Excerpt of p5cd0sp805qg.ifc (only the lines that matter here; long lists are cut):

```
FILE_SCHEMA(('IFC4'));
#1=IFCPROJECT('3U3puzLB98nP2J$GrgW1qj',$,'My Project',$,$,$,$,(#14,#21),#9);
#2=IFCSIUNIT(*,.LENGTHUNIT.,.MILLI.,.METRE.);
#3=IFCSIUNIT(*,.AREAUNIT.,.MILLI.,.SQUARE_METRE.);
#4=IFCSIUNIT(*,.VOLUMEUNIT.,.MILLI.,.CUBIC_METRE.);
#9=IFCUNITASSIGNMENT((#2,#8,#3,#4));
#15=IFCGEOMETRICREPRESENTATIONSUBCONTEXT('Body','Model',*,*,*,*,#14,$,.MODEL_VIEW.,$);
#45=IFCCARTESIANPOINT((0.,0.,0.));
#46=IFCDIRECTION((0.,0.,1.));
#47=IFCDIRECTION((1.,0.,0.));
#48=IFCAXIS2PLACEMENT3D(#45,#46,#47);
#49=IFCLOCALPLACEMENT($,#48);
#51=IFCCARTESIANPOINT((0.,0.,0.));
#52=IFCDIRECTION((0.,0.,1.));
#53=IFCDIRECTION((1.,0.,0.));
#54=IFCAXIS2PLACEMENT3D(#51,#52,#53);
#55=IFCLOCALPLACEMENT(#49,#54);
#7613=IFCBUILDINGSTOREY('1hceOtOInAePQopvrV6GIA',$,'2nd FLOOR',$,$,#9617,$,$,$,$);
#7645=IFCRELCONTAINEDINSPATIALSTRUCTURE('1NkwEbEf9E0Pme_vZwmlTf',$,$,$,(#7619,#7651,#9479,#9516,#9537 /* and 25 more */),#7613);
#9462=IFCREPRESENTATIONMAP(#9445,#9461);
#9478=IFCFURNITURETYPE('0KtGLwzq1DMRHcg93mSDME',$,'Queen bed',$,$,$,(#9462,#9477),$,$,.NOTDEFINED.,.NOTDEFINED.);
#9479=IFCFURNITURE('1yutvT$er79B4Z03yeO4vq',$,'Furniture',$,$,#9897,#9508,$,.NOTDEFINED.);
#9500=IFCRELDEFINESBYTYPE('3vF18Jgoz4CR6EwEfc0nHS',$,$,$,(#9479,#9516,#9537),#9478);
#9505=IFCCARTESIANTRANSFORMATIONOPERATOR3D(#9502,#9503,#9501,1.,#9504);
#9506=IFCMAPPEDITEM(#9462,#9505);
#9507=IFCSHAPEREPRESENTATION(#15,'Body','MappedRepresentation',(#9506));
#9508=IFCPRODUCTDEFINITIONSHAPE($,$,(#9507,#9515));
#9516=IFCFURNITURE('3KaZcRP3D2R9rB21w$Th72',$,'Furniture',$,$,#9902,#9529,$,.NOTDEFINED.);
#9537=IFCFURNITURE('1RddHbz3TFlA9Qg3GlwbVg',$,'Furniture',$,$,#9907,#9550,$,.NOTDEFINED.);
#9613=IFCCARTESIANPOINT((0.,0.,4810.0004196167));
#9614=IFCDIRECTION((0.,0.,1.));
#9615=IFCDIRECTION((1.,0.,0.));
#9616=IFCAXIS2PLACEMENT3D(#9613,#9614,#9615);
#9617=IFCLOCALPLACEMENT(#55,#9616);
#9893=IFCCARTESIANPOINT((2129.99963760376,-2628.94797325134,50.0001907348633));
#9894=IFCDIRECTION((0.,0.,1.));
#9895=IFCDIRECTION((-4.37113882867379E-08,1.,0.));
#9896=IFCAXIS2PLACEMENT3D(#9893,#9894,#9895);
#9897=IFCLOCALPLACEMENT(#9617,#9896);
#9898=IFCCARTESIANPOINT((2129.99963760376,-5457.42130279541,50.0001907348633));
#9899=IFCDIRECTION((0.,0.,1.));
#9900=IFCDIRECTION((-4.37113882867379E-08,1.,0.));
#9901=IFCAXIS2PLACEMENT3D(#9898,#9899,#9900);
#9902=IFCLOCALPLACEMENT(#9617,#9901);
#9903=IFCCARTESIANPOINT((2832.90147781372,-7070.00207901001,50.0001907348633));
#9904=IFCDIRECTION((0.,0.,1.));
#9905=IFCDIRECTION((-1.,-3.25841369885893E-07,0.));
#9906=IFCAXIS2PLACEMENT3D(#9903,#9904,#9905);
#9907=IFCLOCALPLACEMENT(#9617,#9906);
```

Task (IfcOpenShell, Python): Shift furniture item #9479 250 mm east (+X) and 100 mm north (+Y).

```python
import ifcopenshell
import ifcopenshell.api.geometry
import ifcopenshell.util.placement
import ifcopenshell.util.unit

model = ifcopenshell.open("p5cd0sp805qg.ifc")
unit_scale = ifcopenshell.util.unit.calculate_unit_scale(model)

item = model.by_id(9479)
matrix = ifcopenshell.util.placement.get_local_placement(item.ObjectPlacement)
matrix[0, 3] += 0.25 / unit_scale
matrix[1, 3] += 0.1 / unit_scale
ifcopenshell.api.geometry.edit_object_placement(model, product=item, matrix=matrix, is_si=False)

print(ifcopenshell.util.placement.get_local_placement(item.ObjectPlacement).round(3) + 0.0)

model.write("p5cd0sp805qg_v2.ifc")
```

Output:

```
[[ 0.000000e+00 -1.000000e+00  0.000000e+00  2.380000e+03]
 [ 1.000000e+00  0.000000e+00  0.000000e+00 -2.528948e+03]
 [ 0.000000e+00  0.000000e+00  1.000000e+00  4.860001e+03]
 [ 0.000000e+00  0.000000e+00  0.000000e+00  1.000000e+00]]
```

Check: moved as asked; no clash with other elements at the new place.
